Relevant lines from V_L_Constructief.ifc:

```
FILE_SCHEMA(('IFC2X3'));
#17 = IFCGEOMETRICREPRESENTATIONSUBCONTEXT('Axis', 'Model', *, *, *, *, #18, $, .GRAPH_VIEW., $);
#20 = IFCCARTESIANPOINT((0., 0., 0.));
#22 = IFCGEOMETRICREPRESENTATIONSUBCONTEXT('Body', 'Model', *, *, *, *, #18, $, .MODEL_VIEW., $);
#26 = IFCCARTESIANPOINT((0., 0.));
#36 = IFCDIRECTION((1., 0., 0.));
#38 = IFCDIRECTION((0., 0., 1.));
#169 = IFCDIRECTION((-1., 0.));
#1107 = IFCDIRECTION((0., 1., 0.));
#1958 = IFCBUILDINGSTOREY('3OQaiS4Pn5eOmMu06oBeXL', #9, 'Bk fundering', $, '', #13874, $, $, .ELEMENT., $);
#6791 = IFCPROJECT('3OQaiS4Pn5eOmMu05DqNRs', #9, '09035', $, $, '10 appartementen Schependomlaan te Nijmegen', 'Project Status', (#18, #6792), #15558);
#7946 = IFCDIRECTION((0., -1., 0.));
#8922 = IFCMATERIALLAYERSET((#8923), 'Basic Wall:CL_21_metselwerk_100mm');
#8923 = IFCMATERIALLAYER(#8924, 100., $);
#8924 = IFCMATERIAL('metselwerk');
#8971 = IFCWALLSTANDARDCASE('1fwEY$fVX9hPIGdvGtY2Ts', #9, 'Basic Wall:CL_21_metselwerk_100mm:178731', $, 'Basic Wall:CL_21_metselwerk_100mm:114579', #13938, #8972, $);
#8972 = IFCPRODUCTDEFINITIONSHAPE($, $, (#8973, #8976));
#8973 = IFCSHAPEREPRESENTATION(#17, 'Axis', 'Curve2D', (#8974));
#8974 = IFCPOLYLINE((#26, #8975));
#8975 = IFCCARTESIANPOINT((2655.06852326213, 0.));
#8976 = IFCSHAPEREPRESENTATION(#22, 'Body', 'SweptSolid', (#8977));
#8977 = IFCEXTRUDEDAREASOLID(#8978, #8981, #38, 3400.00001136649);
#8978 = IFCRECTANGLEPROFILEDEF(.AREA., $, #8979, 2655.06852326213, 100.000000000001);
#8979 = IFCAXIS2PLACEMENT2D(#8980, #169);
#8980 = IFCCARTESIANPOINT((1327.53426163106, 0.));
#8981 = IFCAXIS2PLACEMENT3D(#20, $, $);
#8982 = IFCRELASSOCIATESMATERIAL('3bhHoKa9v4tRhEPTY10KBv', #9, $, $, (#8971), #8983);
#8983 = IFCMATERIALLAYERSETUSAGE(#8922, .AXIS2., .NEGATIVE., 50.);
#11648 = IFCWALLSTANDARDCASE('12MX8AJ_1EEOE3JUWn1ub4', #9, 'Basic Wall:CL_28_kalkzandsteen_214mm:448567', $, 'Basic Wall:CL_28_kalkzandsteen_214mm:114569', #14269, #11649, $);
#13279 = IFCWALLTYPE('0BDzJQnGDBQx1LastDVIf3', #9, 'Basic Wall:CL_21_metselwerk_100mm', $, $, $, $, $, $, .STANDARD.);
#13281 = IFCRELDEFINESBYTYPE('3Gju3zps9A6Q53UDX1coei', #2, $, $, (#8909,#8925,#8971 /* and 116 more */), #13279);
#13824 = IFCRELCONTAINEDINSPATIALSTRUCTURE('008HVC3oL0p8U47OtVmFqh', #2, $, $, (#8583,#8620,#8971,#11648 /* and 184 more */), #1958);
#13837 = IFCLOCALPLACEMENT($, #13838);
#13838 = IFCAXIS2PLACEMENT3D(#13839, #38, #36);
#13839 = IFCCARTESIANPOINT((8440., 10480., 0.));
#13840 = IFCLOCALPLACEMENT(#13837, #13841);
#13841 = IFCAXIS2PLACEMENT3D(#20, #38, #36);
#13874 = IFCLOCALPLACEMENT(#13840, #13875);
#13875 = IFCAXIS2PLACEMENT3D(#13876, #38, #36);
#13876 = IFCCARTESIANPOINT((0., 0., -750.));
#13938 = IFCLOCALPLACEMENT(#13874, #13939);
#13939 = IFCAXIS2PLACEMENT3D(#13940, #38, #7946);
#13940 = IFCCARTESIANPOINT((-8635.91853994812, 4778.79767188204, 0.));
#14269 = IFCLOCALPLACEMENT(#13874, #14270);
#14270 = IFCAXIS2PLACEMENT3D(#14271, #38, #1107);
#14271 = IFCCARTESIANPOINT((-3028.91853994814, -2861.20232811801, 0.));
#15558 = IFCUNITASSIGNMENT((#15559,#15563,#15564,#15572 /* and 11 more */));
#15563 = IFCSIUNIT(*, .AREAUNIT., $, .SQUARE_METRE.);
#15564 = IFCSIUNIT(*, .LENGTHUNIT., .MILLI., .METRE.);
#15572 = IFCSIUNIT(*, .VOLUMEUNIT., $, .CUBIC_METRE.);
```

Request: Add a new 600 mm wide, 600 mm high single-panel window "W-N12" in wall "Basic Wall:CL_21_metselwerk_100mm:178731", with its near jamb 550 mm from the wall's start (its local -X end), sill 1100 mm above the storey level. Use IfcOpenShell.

```python
import numpy as np
import ifcopenshell
import ifcopenshell.api.feature
import ifcopenshell.api.geometry
import ifcopenshell.api.root
import ifcopenshell.api.spatial
import ifcopenshell.api.type
import ifcopenshell.geom
import ifcopenshell.util.element
import ifcopenshell.util.placement
import ifcopenshell.util.representation
import ifcopenshell.util.shape
import ifcopenshell.util.unit

model = ifcopenshell.open("V_L_Constructief.ifc")
unit_scale = ifcopenshell.util.unit.calculate_unit_scale(model)
settings = ifcopenshell.geom.settings()


def volume(element):
    """Net volume in cubic metres, openings subtracted."""
    shape = ifcopenshell.geom.create_shape(settings, element)
    return ifcopenshell.util.shape.get_volume(shape.geometry)


wall = model.by_guid("1fwEY$fVX9hPIGdvGtY2Ts")
storey = ifcopenshell.util.element.get_container(wall, ifc_class="IfcBuildingStorey")
context = ifcopenshell.util.representation.get_context(model, "Model", "Body", "MODEL_VIEW")
before = volume(wall)

width, height, from_end, sill = 0.6, 0.6, 0.55, 1.1  # metres

# The wall runs along its own X axis, and the end named is its -X end.
wall_shape = ifcopenshell.geom.create_shape(settings, wall)
x, y, z = ifcopenshell.util.shape.get_vertices(wall_shape.geometry).T
start = x.min() + from_end
face, thickness = float(y.min()), float(y.max() - y.min())
wall_matrix = ifcopenshell.util.placement.get_local_placement(wall.ObjectPlacement)
level = ifcopenshell.util.placement.get_local_placement(storey.ObjectPlacement)[2, 3]


def in_wall(x, y):
    """Placement at x, y metres in the wall's axes, at sill height."""
    matrix = wall_matrix.copy()
    matrix[:, 3] = wall_matrix @ np.array([x / unit_scale, y / unit_scale, 0.0, 1.0])
    matrix[2, 3] = level + sill / unit_scale
    return matrix


# Opening: a box that overshoots both wall faces by 50 mm.
opening = ifcopenshell.api.root.create_entity(model, ifc_class="IfcOpeningElement")
box = ifcopenshell.api.geometry.add_wall_representation(
    model, context=context, length=width, height=height, thickness=thickness + 0.1
)
ifcopenshell.api.geometry.assign_representation(model, product=opening, representation=box)
ifcopenshell.api.geometry.edit_object_placement(model, product=opening, matrix=in_wall(start, face - 0.05), is_si=False)
ifcopenshell.api.feature.add_feature(model, feature=opening, element=wall)

window = ifcopenshell.api.root.create_entity(model, ifc_class="IfcWindow", name="W-N12")
window.OverallWidth, window.OverallHeight = width / unit_scale, height / unit_scale
body = ifcopenshell.api.geometry.add_window_representation(
    model,
    context=context,
    overall_width=window.OverallWidth,
    overall_height=window.OverallHeight,
    partition_type="SINGLE_PANEL",
)
ifcopenshell.api.geometry.assign_representation(model, product=window, representation=body)
ifcopenshell.api.spatial.assign_container(model, products=[window], relating_structure=storey)
fills = ifcopenshell.api.feature.add_filling(model, opening=opening, element=window)
fills.OwnerHistory = window.OwnerHistory  # required in IFC2X3

# IFC2X3 keeps the operation on the window style.
style = ifcopenshell.api.root.create_entity(model, ifc_class="IfcWindowStyle", name="W-N12")
style.OperationType, style.ConstructionType = "SINGLE_PANEL", "NOTDEFINED"
style.ParameterTakesPrecedence = style.Sizeable = False
ifcopenshell.api.type.assign_type(model, related_objects=[window], relating_type=style)

# Centre the window in the wall's thickness.
ifcopenshell.api.geometry.edit_object_placement(model, product=window, matrix=in_wall(start, face), is_si=False)
window_shape = ifcopenshell.geom.create_shape(settings, window)
depth = ifcopenshell.util.shape.get_vertices(window_shape.geometry)[:, 1]
offset = face + thickness / 2 - (depth.min() + depth.max()) / 2
ifcopenshell.api.geometry.edit_object_placement(model, product=window, matrix=in_wall(start, offset), is_si=False)

after = volume(wall)

print(f"wall volume {before:.3f} -> {after:.3f} m3")

model.write("V_L_Constructief_rev.ifc")
```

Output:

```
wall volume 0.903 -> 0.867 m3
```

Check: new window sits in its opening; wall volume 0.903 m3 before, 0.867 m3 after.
